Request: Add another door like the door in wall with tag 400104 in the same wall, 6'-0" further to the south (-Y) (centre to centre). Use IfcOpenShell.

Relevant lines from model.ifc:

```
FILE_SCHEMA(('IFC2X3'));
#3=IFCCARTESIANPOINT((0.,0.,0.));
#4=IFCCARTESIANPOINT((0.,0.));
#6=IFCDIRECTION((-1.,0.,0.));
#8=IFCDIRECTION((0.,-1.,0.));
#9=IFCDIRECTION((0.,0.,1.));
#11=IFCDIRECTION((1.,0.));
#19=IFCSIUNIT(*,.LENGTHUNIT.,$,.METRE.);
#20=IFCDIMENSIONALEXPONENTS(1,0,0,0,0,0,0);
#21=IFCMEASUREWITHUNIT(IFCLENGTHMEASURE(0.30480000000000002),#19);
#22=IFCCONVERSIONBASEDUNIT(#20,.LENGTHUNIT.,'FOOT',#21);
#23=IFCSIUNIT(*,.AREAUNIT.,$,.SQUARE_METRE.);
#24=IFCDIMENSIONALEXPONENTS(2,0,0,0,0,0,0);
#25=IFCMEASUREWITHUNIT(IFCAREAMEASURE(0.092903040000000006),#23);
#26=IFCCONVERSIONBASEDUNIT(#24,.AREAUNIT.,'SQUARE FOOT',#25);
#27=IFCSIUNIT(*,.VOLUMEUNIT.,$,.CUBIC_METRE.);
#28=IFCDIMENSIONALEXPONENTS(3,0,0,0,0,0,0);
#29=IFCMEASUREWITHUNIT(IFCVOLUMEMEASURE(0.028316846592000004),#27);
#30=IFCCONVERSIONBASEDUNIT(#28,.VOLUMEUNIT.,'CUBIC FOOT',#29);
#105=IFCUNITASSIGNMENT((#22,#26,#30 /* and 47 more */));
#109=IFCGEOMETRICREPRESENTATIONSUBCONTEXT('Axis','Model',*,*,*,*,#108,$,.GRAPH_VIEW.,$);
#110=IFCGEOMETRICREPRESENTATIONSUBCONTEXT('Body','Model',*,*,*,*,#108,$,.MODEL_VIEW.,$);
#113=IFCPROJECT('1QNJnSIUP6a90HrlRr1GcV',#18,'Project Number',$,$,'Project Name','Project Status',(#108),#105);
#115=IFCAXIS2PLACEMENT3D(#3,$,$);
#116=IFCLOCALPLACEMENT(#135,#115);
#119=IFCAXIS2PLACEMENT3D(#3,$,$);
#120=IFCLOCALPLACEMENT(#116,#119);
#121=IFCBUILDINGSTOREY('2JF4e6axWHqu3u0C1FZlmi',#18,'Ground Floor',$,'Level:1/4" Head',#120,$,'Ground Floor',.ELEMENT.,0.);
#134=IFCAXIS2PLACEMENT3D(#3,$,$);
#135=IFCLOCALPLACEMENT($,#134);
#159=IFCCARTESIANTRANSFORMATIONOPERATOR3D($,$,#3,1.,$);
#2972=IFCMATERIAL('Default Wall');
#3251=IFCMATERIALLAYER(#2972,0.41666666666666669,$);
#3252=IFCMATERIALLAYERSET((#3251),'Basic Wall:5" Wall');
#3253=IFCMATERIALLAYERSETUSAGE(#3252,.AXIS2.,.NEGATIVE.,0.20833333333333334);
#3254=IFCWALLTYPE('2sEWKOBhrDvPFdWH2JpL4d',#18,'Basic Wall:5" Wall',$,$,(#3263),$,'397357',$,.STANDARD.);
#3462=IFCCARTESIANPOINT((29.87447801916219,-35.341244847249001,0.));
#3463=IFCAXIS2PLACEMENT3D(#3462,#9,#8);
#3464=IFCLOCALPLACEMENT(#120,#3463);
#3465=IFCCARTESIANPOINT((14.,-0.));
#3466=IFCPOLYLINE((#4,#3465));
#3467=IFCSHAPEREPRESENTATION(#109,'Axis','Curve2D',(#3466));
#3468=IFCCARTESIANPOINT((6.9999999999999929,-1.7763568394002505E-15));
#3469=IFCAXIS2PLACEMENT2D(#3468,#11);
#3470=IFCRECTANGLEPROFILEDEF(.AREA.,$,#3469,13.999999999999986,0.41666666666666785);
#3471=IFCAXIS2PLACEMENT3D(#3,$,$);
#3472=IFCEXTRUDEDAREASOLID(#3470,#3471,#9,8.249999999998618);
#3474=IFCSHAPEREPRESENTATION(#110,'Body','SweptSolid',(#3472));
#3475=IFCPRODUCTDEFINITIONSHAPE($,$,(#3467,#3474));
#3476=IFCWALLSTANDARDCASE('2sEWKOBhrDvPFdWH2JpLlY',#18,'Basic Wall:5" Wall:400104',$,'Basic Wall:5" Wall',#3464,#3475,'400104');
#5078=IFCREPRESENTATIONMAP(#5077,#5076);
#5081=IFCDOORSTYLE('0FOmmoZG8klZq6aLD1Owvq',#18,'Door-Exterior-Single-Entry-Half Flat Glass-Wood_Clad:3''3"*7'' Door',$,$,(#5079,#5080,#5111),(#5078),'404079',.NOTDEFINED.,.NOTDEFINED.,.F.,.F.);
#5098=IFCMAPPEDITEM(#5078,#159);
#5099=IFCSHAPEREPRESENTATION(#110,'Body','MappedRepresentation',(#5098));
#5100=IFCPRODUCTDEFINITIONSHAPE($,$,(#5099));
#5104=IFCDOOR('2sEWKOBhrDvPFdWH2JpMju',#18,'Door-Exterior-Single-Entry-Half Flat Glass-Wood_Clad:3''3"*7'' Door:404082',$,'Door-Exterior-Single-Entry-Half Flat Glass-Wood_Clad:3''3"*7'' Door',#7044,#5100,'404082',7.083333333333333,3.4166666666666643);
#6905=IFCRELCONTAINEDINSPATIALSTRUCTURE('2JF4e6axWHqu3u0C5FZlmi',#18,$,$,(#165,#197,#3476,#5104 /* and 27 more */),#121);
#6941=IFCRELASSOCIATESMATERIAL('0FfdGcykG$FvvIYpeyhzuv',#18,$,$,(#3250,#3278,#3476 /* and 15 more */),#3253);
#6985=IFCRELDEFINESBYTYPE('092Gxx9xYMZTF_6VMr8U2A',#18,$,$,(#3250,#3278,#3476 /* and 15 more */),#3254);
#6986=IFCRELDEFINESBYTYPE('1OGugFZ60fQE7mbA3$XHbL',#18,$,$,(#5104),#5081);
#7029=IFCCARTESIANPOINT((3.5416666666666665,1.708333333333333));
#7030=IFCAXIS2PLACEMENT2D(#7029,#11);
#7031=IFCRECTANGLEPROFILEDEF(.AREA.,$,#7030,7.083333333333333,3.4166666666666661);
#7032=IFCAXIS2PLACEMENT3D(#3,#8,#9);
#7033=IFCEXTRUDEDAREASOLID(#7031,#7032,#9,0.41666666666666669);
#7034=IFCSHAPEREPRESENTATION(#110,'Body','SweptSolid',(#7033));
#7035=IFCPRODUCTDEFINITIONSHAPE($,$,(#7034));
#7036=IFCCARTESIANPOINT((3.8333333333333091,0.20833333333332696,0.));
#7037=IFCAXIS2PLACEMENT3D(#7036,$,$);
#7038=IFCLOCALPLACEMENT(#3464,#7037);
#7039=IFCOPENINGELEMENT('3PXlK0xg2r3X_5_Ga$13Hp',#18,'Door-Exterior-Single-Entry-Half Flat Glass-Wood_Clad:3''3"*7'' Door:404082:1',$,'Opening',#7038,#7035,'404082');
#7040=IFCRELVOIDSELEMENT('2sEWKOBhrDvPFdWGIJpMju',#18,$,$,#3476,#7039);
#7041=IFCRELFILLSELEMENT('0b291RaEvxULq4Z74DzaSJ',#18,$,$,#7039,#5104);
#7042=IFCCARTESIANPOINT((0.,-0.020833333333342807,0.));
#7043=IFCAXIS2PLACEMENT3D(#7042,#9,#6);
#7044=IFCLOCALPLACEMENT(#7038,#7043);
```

```python
import ifcopenshell
import ifcopenshell.api.feature
import ifcopenshell.api.geometry
import ifcopenshell.api.root
import ifcopenshell.geom
import ifcopenshell.util.element
import ifcopenshell.util.placement
import ifcopenshell.util.shape
import ifcopenshell.util.unit

model = ifcopenshell.open("model.ifc")
unit_scale = ifcopenshell.util.unit.calculate_unit_scale(model)
settings = ifcopenshell.geom.settings()


def volume(element):
    """Net volume in cubic metres, openings subtracted."""
    shape = ifcopenshell.geom.create_shape(settings, element)
    return ifcopenshell.util.shape.get_volume(shape.geometry)


def reuse_history(source, copy):
    """copy_class also copies each property set's owner history, people and application; keep the originals."""
    for rel in copy.IsDefinedBy:
        if rel.is_a("IfcRelDefinesByProperties") and (history := rel.RelatingPropertyDefinition.OwnerHistory):
            rel.RelatingPropertyDefinition.OwnerHistory = source.OwnerHistory
            ifcopenshell.util.element.remove_deep2(model, history)


door = model.by_id(5104)
opening = door.FillsVoids[0].RelatingOpeningElement
wall = opening.VoidsElements[0].RelatingBuildingElement
before = volume(wall)
shift = ifcopenshell.util.placement.get_local_placement(wall.ObjectPlacement)[:3, 0] * 72 * 0.0254 / unit_scale

# copy_class copies the void relationship, type, container and properties, but no geometry.
new_opening = ifcopenshell.api.root.copy_class(model, product=opening)
new_opening.Representation = ifcopenshell.util.element.copy_deep(
    model, opening.Representation, exclude=["IfcGeometricRepresentationContext", "IfcRepresentationMap"]
)
new_opening.Name = 'Door-Exterior-Single-Entry-Half Flat Glass-Wood_Clad:3\'3"*7\' Door'
new_opening.Tag = None
new_door = ifcopenshell.api.root.copy_class(model, product=door)
new_door.Representation = ifcopenshell.util.element.copy_deep(
    model, door.Representation, exclude=["IfcGeometricRepresentationContext", "IfcRepresentationMap"]
)
new_door.Name = 'Door-Exterior-Single-Entry-Half Flat Glass-Wood_Clad:3\'3"*7\' Door'
new_door.Tag = None
reuse_history(door, new_door)
fills = ifcopenshell.api.feature.add_filling(model, opening=new_opening, element=new_door)
fills.OwnerHistory = new_door.OwnerHistory  # required in IFC2X3

for old, new in ((opening, new_opening), (door, new_door)):
    matrix = ifcopenshell.util.placement.get_local_placement(old.ObjectPlacement)
    matrix[:3, 3] += shift
    ifcopenshell.api.geometry.edit_object_placement(model, product=new, matrix=matrix, is_si=False)

after = volume(wall)

print(f"wall volume {before:.3f} -> {after:.3f} m3")

model.write("model_updated.ifc")
```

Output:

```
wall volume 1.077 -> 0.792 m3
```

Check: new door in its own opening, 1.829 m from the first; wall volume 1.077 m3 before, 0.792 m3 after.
